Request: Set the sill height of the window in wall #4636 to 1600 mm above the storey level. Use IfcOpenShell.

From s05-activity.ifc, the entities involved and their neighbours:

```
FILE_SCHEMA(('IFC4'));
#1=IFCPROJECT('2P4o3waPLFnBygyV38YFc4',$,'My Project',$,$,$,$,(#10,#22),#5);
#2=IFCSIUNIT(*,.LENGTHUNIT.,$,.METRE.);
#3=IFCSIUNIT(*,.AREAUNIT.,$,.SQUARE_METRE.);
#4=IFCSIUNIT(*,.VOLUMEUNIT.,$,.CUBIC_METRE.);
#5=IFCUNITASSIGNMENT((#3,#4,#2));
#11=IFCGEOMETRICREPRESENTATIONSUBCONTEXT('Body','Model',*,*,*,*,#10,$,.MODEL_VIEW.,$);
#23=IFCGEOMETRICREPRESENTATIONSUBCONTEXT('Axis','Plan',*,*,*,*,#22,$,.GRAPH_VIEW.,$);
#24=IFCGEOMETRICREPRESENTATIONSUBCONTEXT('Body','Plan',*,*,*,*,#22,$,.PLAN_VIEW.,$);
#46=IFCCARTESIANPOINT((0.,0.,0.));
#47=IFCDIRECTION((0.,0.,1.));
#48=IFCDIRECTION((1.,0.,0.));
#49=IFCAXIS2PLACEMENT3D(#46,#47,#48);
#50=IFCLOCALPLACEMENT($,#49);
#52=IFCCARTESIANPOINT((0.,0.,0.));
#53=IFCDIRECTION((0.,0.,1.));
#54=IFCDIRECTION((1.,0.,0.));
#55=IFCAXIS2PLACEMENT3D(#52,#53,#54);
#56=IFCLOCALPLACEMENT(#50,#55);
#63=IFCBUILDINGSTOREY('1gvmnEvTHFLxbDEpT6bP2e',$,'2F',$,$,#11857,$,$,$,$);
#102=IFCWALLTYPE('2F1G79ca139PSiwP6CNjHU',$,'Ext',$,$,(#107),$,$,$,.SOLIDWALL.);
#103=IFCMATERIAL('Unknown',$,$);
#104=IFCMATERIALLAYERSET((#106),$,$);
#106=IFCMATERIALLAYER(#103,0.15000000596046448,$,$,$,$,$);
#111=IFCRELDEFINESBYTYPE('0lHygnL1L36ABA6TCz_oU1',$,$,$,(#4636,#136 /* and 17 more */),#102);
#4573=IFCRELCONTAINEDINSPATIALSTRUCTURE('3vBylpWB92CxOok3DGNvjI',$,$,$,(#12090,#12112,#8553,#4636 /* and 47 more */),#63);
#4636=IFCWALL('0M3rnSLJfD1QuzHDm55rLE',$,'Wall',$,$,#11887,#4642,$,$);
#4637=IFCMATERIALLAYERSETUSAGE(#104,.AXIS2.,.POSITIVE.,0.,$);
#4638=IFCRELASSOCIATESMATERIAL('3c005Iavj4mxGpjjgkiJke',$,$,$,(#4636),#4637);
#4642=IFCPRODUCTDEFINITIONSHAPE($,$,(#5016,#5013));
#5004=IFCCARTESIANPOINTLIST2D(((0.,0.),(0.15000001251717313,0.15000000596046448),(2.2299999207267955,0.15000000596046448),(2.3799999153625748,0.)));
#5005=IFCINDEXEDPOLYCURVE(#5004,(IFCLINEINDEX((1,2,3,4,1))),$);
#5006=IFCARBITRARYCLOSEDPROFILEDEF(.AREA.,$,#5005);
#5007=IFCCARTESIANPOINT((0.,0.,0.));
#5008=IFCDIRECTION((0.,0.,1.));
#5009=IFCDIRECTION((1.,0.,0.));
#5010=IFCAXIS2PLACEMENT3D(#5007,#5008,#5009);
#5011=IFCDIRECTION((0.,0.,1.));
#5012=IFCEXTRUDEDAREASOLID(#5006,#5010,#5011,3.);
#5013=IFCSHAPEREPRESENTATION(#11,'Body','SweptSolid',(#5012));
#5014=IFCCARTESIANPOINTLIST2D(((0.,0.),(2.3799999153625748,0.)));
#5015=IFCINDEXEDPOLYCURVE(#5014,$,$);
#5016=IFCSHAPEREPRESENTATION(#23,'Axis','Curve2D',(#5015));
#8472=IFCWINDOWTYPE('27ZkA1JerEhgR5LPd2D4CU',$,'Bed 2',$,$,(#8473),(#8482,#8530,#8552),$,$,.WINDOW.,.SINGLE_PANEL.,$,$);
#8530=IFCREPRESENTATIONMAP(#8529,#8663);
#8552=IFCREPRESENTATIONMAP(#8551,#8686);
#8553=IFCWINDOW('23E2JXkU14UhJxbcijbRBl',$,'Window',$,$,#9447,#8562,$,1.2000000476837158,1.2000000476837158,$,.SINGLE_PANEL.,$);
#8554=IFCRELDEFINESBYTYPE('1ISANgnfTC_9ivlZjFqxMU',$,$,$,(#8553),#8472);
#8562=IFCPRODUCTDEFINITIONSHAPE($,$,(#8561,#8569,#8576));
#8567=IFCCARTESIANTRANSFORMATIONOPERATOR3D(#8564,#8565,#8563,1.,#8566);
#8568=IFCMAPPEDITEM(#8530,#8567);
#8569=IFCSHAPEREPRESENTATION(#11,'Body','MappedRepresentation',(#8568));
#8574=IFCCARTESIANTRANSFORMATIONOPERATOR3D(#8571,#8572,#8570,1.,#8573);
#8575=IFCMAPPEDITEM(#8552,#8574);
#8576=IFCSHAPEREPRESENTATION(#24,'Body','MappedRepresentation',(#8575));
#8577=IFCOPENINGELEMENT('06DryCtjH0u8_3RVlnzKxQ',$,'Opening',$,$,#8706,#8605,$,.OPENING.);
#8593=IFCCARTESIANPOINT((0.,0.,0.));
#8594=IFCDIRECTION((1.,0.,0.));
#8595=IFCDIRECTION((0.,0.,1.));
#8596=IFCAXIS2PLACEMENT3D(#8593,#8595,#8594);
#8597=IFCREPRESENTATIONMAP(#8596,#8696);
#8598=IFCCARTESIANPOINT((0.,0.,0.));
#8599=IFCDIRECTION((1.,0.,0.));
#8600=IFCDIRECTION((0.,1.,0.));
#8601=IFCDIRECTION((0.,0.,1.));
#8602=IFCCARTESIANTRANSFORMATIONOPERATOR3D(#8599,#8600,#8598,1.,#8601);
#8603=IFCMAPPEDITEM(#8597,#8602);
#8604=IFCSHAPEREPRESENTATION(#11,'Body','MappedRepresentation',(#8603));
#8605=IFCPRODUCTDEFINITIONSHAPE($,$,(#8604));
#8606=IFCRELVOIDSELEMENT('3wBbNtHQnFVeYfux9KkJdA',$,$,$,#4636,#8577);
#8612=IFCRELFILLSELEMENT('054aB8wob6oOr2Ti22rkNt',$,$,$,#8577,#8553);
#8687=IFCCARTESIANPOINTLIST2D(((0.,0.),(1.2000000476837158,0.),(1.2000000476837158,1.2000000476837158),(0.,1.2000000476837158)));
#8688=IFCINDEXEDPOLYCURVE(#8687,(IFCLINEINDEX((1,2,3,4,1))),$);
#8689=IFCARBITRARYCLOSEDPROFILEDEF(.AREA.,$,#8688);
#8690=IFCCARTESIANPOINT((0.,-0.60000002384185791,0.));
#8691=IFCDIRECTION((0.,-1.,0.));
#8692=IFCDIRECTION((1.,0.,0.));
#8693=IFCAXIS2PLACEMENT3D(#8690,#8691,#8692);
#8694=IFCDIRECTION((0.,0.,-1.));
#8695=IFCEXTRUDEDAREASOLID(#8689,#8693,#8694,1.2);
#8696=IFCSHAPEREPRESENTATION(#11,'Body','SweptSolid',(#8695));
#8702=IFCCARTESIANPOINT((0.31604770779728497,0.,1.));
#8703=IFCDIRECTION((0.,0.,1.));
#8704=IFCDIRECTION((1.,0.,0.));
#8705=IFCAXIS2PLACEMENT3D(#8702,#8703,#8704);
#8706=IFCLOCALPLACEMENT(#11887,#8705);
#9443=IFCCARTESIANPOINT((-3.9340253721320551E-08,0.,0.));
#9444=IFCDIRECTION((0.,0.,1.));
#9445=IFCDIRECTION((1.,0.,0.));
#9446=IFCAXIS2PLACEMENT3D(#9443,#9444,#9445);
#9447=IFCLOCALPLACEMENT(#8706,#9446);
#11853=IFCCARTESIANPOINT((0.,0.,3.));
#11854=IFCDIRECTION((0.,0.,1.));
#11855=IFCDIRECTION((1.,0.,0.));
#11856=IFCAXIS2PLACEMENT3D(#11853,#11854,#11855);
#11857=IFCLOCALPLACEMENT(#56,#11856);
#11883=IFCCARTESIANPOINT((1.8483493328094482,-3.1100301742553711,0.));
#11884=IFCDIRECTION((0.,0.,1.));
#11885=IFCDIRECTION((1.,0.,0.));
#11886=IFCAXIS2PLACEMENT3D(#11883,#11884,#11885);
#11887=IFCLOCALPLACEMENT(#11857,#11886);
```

```python
import numpy as np
import ifcopenshell
import ifcopenshell.api.geometry
import ifcopenshell.geom
import ifcopenshell.util.element
import ifcopenshell.util.placement
import ifcopenshell.util.shape
import ifcopenshell.util.unit

model = ifcopenshell.open("s05-activity.ifc")
unit_scale = ifcopenshell.util.unit.calculate_unit_scale(model)

window = model.by_guid("23E2JXkU14UhJxbcijbRBl")
opening = window.FillsVoids[0].RelatingOpeningElement
storey = ifcopenshell.util.element.get_container(window, ifc_class="IfcBuildingStorey")
level = ifcopenshell.util.placement.get_local_placement(storey.ObjectPlacement)[2, 3]

# The opening's origin need not be at the sill, so measure its lowest point.
shape = ifcopenshell.geom.create_shape(ifcopenshell.geom.settings(), opening)
bottom = ifcopenshell.util.shape.get_shape_bottom_elevation(shape, shape.geometry) / unit_scale
dz = level + 1.6 / unit_scale - bottom

shift = np.array([0.0, 0.0, dz])
# The window is placed relative to its opening, so it follows when the opening moves.
matrix = ifcopenshell.util.placement.get_local_placement(opening.ObjectPlacement)
matrix[:3, 3] += shift
ifcopenshell.api.geometry.edit_object_placement(
    model, product=opening, matrix=matrix, is_si=False, should_transform_children=True
)

print(f"moved by {dz * unit_scale:+.3f} m")

model.write("s05-activity_updated.ifc")
```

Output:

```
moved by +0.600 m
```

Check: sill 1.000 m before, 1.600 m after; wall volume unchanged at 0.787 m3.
